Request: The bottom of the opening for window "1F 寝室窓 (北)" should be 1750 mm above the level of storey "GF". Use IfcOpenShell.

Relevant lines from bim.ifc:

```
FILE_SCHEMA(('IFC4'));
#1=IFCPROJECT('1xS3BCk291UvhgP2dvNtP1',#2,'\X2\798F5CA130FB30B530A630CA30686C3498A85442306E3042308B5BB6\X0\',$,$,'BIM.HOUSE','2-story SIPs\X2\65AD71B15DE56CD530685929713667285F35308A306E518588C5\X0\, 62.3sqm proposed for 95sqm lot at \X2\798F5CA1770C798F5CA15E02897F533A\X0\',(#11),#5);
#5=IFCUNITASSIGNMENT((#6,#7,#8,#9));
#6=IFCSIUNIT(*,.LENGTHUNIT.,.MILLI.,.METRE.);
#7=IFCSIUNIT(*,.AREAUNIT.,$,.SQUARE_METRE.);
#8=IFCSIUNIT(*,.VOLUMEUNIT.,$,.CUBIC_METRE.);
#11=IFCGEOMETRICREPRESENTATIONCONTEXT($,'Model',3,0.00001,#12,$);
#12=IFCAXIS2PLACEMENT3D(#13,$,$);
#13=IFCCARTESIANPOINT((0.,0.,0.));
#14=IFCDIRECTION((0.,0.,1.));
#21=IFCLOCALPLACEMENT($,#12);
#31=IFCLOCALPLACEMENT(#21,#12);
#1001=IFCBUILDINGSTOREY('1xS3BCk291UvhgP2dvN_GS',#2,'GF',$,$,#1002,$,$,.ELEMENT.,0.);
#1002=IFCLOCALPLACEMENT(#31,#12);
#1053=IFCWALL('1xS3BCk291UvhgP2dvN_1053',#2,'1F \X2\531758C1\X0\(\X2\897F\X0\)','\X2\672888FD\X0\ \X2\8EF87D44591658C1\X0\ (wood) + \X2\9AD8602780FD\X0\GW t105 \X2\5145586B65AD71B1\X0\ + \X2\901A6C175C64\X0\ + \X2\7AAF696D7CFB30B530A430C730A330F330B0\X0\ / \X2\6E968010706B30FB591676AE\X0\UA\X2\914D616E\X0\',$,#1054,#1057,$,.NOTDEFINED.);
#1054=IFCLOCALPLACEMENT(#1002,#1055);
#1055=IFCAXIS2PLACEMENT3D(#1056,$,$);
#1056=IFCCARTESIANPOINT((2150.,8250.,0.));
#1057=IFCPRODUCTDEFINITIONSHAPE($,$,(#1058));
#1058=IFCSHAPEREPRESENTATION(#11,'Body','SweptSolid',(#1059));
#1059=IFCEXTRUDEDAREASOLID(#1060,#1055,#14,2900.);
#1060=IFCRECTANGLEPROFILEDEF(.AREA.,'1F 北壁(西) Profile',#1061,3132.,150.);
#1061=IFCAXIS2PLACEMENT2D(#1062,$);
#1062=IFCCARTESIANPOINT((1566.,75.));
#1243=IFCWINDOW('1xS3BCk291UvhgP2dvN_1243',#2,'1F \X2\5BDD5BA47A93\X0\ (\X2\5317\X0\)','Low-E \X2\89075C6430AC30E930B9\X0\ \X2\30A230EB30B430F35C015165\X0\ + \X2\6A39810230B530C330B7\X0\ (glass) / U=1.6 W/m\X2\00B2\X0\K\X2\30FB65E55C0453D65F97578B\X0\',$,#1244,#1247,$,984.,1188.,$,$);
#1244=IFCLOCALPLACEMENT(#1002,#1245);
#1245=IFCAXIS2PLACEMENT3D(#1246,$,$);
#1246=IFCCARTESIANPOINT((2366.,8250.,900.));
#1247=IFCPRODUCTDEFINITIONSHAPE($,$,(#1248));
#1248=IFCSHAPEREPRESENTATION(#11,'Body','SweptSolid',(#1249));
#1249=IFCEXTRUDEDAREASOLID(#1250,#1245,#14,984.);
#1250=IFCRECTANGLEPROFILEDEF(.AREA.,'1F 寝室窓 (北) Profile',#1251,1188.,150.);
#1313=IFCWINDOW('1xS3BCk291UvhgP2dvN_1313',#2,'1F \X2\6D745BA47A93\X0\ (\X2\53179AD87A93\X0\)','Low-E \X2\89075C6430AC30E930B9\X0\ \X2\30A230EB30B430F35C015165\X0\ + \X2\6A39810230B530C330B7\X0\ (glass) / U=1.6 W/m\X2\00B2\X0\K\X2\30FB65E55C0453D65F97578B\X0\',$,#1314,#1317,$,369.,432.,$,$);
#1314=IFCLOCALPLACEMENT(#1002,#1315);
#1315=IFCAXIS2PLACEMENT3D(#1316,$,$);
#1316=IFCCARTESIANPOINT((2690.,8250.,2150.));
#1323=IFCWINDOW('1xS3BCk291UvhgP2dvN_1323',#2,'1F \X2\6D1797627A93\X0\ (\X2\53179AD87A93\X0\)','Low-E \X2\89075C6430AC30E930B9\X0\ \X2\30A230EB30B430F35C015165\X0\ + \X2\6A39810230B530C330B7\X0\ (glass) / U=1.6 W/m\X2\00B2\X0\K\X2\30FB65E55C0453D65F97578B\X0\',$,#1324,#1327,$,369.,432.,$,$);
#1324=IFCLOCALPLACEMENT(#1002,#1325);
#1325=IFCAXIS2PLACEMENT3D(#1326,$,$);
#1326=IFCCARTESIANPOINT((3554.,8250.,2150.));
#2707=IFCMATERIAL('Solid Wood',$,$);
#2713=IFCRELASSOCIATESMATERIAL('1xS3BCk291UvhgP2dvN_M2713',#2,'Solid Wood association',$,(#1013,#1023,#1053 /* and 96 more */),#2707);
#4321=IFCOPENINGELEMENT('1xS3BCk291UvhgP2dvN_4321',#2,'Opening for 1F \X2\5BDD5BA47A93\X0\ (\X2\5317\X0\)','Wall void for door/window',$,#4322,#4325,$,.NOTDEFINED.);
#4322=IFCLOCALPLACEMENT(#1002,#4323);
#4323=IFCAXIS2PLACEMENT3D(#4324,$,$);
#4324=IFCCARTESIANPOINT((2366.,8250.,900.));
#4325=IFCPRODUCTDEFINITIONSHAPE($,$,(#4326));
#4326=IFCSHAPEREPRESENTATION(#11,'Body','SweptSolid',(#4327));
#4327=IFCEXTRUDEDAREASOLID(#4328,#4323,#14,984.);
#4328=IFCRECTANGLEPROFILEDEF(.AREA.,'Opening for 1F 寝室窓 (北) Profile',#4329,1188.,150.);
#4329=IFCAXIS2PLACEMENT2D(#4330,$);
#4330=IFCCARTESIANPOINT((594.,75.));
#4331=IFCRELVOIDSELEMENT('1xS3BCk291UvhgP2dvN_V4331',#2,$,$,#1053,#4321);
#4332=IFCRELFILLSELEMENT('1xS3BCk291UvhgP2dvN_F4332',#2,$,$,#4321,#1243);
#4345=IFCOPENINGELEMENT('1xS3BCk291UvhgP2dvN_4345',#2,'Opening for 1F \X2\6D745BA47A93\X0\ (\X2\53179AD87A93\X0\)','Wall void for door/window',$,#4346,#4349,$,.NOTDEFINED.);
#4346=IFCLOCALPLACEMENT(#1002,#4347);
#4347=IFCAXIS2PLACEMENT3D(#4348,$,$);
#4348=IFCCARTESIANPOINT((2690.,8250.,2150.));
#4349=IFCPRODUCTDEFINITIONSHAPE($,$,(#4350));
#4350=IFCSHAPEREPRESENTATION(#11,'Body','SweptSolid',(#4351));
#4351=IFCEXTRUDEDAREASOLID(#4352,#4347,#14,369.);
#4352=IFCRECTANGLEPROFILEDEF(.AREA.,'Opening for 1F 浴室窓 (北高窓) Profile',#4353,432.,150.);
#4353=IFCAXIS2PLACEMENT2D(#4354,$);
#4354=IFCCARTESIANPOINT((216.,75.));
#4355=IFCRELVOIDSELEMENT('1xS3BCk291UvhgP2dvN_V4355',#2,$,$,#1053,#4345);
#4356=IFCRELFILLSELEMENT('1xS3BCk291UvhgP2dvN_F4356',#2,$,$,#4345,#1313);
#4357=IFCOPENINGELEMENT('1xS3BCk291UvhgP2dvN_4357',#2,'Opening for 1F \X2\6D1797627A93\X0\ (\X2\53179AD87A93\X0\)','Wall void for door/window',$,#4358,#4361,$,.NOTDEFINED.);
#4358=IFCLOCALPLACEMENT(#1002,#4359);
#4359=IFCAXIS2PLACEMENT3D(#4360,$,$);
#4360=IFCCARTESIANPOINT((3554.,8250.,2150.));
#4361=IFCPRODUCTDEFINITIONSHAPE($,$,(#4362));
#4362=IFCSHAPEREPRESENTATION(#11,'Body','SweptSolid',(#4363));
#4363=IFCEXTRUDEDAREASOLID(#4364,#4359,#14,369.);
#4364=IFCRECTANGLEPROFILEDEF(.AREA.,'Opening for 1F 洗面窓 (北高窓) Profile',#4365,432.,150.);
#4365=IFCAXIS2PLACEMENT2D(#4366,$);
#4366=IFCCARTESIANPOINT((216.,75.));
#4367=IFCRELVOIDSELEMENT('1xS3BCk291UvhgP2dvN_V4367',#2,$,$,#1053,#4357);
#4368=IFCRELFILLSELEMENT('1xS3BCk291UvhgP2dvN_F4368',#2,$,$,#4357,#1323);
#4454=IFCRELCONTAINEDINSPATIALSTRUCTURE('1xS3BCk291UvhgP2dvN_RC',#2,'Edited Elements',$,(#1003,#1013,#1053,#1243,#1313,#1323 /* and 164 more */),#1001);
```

```python
import numpy as np
import ifcopenshell
import ifcopenshell.api.geometry
import ifcopenshell.geom
import ifcopenshell.util.element
import ifcopenshell.util.placement
import ifcopenshell.util.shape
import ifcopenshell.util.unit

model = ifcopenshell.open("bim.ifc")
unit_scale = ifcopenshell.util.unit.calculate_unit_scale(model)

window = model.by_guid("1xS3BCk291UvhgP2dvN_1243")
opening = window.FillsVoids[0].RelatingOpeningElement
storey = ifcopenshell.util.element.get_container(window, ifc_class="IfcBuildingStorey")
level = ifcopenshell.util.placement.get_local_placement(storey.ObjectPlacement)[2, 3]

# The opening's origin need not be at the sill, so measure its lowest point.
shape = ifcopenshell.geom.create_shape(ifcopenshell.geom.settings(), opening)
bottom = ifcopenshell.util.shape.get_shape_bottom_elevation(shape, shape.geometry) / unit_scale
dz = level + 1750.0 - bottom

shift = np.array([0.0, 0.0, dz])
# The window is not placed relative to its opening, so move both.
for product in (opening, window):
    matrix = ifcopenshell.util.placement.get_local_placement(product.ObjectPlacement)
    matrix[:3, 3] += shift
    ifcopenshell.api.geometry.edit_object_placement(model, product=product, matrix=matrix, is_si=False)

print(f"moved by {dz * unit_scale:+.3f} m")

model.write("bim_rev.ifc")
```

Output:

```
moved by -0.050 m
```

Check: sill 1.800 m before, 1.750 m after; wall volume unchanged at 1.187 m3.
